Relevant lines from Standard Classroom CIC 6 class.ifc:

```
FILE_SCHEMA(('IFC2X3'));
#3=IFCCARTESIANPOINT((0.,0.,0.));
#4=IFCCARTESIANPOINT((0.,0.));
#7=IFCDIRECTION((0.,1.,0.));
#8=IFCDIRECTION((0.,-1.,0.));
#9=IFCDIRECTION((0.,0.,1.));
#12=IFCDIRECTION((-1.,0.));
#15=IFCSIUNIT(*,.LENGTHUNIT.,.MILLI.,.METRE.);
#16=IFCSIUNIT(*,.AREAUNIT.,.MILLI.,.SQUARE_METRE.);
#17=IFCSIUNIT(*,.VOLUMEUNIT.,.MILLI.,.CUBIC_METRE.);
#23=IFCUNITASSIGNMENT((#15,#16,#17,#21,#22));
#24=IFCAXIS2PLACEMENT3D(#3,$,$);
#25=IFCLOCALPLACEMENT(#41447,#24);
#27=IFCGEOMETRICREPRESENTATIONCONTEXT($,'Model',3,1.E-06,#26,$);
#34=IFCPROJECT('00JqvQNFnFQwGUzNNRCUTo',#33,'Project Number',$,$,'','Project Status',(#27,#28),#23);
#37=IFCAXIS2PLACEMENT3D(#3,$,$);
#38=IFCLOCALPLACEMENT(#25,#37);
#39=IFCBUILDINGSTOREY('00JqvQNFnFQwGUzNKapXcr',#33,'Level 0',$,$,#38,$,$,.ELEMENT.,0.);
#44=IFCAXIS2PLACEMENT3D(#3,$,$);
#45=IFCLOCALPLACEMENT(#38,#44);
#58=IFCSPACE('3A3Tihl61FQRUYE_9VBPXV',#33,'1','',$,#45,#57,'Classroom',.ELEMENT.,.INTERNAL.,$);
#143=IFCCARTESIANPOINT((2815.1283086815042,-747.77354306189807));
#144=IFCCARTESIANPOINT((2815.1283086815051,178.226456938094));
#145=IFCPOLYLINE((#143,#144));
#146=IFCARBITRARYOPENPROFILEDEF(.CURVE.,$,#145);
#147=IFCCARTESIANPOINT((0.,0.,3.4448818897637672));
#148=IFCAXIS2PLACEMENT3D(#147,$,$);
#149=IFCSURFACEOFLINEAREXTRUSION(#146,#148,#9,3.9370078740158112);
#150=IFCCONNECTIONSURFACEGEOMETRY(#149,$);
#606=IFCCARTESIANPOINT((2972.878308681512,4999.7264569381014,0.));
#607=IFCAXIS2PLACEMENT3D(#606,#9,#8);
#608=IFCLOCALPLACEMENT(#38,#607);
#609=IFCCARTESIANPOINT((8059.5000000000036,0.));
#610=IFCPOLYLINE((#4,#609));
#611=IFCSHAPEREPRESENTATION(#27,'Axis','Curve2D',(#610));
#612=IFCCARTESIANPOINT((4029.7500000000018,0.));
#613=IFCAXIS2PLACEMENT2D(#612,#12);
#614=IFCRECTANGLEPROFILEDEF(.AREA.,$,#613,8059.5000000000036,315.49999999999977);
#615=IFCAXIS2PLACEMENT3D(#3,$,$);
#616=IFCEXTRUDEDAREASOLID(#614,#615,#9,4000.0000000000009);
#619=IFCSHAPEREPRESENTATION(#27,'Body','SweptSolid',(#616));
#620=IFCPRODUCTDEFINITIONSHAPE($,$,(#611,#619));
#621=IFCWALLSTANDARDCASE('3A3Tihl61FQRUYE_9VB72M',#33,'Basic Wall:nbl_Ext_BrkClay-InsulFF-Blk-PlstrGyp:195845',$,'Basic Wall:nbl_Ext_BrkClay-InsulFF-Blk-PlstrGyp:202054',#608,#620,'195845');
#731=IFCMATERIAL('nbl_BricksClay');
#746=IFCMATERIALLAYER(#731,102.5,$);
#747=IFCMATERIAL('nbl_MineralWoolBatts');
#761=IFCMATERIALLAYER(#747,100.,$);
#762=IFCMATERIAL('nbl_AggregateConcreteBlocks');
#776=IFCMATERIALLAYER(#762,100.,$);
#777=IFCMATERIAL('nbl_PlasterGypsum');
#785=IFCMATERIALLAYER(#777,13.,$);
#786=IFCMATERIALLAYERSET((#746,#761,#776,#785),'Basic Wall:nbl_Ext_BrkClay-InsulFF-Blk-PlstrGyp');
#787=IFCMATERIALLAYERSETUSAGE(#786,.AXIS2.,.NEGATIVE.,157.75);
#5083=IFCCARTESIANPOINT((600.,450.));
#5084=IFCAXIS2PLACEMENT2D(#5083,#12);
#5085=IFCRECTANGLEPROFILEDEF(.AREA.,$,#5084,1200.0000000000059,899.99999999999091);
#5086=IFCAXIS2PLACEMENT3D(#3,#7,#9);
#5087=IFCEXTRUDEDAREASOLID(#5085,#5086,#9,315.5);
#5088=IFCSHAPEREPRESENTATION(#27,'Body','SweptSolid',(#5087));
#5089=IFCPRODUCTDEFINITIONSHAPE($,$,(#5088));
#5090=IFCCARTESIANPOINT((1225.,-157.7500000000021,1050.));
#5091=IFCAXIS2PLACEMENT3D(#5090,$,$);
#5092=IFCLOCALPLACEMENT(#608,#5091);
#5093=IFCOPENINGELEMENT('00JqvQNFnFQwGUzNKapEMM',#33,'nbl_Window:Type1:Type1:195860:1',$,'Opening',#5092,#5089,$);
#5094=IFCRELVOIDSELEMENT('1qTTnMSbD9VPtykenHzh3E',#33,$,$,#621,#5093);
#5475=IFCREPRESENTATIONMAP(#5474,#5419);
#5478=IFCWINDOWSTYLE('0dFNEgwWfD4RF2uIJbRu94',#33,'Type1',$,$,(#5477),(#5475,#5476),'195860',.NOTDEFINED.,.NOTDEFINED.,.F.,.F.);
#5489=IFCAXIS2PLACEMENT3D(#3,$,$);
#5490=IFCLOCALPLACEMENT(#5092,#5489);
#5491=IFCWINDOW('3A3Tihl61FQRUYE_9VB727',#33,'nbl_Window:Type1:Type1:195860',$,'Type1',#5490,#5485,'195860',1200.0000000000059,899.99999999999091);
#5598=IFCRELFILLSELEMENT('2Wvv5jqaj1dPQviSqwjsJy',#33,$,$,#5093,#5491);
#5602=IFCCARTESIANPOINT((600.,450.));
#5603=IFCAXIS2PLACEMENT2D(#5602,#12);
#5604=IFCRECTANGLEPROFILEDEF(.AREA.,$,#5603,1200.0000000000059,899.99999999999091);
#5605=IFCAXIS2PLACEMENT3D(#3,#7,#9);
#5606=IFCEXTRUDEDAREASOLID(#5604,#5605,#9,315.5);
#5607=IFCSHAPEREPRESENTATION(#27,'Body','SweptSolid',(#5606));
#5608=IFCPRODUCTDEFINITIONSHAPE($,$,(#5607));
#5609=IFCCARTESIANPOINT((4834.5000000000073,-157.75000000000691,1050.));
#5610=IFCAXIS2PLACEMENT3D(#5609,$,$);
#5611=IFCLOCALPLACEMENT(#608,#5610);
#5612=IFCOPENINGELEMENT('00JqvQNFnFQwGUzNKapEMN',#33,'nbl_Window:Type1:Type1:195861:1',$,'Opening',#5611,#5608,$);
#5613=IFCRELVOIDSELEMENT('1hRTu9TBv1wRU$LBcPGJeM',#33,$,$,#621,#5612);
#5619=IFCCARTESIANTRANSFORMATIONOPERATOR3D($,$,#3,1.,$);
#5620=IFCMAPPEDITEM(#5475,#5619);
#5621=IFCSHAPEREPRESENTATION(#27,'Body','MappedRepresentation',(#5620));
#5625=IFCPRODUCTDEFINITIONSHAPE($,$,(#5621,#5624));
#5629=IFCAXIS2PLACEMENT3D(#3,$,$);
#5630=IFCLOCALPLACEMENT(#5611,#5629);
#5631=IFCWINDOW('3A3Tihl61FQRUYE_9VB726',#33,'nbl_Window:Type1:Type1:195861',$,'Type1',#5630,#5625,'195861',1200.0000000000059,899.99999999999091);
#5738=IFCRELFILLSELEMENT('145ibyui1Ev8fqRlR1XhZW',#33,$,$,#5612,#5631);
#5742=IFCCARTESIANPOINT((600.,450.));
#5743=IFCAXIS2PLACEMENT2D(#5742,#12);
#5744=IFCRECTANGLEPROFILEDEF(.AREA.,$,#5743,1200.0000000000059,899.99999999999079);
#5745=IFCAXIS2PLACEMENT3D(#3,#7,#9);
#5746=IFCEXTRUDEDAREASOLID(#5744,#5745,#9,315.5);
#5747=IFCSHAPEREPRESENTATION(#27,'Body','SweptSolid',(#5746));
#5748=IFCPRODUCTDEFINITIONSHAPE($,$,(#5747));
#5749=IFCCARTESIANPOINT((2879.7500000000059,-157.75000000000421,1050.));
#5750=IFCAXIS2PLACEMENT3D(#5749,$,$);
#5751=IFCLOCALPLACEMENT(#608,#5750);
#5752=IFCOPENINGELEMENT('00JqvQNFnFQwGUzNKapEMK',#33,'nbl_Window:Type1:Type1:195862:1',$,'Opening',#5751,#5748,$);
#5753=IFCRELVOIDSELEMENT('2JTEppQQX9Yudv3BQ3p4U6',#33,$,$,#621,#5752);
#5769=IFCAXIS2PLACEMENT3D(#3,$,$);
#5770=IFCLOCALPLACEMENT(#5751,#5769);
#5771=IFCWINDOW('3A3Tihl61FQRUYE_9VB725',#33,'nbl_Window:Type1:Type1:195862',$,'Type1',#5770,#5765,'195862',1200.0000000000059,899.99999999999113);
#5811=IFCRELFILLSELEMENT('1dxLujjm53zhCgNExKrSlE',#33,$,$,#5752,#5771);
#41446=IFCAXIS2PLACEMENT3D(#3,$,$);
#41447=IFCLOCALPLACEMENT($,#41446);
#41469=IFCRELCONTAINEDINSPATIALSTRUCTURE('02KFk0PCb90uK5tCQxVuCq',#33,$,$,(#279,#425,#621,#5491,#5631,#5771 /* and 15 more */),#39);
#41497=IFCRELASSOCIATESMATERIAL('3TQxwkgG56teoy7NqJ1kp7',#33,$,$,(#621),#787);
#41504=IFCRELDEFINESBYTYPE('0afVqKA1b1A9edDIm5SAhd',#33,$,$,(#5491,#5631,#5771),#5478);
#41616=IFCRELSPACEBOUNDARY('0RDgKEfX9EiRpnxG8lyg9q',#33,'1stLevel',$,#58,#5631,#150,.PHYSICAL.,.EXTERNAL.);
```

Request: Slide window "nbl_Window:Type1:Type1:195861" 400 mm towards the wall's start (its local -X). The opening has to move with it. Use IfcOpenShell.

```python
import numpy as np
import ifcopenshell
import ifcopenshell.api.geometry
import ifcopenshell.util.placement
import ifcopenshell.util.unit

model = ifcopenshell.open("Standard Classroom CIC 6 class.ifc")
unit_scale = ifcopenshell.util.unit.calculate_unit_scale(model)

window = model.by_guid("3A3Tihl61FQRUYE_9VB726")
opening = window.FillsVoids[0].RelatingOpeningElement
wall = opening.VoidsElements[0].RelatingBuildingElement

wall_matrix = ifcopenshell.util.placement.get_local_placement(wall.ObjectPlacement)
shift = wall_matrix[:3, 0] * -0.4 / unit_scale
before = ifcopenshell.util.placement.get_local_placement(window.ObjectPlacement)[:3, 3].copy()

# The window is placed relative to its opening, so it follows when the opening moves.
matrix = ifcopenshell.util.placement.get_local_placement(opening.ObjectPlacement)
matrix[:3, 3] += shift
ifcopenshell.api.geometry.edit_object_placement(
    model, product=opening, matrix=matrix, is_si=False, should_transform_children=True
)

# Space boundary surfaces are stored in each space's coordinates; move them too.
for rel in window.ProvidesBoundaries:
    if not rel.ConnectionGeometry:
        continue
    surface = rel.ConnectionGeometry.SurfaceOnRelatingElement
    space_matrix = ifcopenshell.util.placement.get_local_placement(rel.RelatingSpace.ObjectPlacement)
    point = np.array(surface.Position.Location.Coordinates) + space_matrix[:3, :3].T @ shift
    surface.Position = model.createIfcAxis2Placement3D(
        model.createIfcCartesianPoint(point.tolist()), surface.Position.Axis, surface.Position.RefDirection
    )

after = ifcopenshell.util.placement.get_local_placement(window.ObjectPlacement)[:3, 3]
print("window moved by", (after - before).round(3) + 0.0)

model.write("Standard Classroom CIC 6 class_v2.ifc")
```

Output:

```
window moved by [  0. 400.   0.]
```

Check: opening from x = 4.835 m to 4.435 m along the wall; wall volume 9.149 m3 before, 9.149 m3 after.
